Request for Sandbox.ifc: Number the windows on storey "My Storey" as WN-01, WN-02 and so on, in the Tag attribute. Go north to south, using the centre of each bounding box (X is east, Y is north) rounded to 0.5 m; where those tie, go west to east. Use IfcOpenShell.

First a look at what the model holds.

```python
import ifcopenshell
import ifcopenshell.util.element
import ifcopenshell.util.placement

model = ifcopenshell.open("Sandbox.ifc")
print(model.schema)
storey = next(s for s in model.by_type("IfcBuildingStorey") if s.Name == "My Storey")
windows = [e for e in ifcopenshell.util.element.get_decomposition(storey) if e.is_a("IfcWindow")]
for e in sorted(windows, key=lambda e: e.id()):
    origin = ifcopenshell.util.placement.get_local_placement(e.ObjectPlacement)[:3, 3]
    print(e.id(), e.Tag, e.Name, origin.round(2) + 0.0, sep=" | ")
```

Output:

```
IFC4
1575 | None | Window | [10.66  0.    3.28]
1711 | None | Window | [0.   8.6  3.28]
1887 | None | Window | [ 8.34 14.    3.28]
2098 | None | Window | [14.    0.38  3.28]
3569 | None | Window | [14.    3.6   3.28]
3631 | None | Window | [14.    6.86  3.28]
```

```python
import ifcopenshell
import ifcopenshell.geom
import ifcopenshell.util.element
import ifcopenshell.util.shape

model = ifcopenshell.open("Sandbox.ifc")
settings = ifcopenshell.geom.settings()
settings.set("use-world-coords", True)


def centre(element):
    shape = ifcopenshell.geom.create_shape(settings, element)
    return ifcopenshell.util.shape.get_bbox_centroid(shape.geometry)


storey = next(s for s in model.by_type("IfcBuildingStorey") if s.Name == "My Storey")
windows = [e for e in ifcopenshell.util.element.get_decomposition(storey) if e.is_a("IfcWindow")]

# Insertion points can sit at a corner or the storey origin, so sort by the geometry (in metres).
centres = {e: centre(e) for e in windows}
windows.sort(key=lambda e: (-round(centres[e][1] / 0.5), centres[e][0]))

for i, e in enumerate(windows, start=1):
    number = f"WN-{i:02d}"
    e.Tag = number
    print(e.id(), number)

model.write("Sandbox-out.ifc")
```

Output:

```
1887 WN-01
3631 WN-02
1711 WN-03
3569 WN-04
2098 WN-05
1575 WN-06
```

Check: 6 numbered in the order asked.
